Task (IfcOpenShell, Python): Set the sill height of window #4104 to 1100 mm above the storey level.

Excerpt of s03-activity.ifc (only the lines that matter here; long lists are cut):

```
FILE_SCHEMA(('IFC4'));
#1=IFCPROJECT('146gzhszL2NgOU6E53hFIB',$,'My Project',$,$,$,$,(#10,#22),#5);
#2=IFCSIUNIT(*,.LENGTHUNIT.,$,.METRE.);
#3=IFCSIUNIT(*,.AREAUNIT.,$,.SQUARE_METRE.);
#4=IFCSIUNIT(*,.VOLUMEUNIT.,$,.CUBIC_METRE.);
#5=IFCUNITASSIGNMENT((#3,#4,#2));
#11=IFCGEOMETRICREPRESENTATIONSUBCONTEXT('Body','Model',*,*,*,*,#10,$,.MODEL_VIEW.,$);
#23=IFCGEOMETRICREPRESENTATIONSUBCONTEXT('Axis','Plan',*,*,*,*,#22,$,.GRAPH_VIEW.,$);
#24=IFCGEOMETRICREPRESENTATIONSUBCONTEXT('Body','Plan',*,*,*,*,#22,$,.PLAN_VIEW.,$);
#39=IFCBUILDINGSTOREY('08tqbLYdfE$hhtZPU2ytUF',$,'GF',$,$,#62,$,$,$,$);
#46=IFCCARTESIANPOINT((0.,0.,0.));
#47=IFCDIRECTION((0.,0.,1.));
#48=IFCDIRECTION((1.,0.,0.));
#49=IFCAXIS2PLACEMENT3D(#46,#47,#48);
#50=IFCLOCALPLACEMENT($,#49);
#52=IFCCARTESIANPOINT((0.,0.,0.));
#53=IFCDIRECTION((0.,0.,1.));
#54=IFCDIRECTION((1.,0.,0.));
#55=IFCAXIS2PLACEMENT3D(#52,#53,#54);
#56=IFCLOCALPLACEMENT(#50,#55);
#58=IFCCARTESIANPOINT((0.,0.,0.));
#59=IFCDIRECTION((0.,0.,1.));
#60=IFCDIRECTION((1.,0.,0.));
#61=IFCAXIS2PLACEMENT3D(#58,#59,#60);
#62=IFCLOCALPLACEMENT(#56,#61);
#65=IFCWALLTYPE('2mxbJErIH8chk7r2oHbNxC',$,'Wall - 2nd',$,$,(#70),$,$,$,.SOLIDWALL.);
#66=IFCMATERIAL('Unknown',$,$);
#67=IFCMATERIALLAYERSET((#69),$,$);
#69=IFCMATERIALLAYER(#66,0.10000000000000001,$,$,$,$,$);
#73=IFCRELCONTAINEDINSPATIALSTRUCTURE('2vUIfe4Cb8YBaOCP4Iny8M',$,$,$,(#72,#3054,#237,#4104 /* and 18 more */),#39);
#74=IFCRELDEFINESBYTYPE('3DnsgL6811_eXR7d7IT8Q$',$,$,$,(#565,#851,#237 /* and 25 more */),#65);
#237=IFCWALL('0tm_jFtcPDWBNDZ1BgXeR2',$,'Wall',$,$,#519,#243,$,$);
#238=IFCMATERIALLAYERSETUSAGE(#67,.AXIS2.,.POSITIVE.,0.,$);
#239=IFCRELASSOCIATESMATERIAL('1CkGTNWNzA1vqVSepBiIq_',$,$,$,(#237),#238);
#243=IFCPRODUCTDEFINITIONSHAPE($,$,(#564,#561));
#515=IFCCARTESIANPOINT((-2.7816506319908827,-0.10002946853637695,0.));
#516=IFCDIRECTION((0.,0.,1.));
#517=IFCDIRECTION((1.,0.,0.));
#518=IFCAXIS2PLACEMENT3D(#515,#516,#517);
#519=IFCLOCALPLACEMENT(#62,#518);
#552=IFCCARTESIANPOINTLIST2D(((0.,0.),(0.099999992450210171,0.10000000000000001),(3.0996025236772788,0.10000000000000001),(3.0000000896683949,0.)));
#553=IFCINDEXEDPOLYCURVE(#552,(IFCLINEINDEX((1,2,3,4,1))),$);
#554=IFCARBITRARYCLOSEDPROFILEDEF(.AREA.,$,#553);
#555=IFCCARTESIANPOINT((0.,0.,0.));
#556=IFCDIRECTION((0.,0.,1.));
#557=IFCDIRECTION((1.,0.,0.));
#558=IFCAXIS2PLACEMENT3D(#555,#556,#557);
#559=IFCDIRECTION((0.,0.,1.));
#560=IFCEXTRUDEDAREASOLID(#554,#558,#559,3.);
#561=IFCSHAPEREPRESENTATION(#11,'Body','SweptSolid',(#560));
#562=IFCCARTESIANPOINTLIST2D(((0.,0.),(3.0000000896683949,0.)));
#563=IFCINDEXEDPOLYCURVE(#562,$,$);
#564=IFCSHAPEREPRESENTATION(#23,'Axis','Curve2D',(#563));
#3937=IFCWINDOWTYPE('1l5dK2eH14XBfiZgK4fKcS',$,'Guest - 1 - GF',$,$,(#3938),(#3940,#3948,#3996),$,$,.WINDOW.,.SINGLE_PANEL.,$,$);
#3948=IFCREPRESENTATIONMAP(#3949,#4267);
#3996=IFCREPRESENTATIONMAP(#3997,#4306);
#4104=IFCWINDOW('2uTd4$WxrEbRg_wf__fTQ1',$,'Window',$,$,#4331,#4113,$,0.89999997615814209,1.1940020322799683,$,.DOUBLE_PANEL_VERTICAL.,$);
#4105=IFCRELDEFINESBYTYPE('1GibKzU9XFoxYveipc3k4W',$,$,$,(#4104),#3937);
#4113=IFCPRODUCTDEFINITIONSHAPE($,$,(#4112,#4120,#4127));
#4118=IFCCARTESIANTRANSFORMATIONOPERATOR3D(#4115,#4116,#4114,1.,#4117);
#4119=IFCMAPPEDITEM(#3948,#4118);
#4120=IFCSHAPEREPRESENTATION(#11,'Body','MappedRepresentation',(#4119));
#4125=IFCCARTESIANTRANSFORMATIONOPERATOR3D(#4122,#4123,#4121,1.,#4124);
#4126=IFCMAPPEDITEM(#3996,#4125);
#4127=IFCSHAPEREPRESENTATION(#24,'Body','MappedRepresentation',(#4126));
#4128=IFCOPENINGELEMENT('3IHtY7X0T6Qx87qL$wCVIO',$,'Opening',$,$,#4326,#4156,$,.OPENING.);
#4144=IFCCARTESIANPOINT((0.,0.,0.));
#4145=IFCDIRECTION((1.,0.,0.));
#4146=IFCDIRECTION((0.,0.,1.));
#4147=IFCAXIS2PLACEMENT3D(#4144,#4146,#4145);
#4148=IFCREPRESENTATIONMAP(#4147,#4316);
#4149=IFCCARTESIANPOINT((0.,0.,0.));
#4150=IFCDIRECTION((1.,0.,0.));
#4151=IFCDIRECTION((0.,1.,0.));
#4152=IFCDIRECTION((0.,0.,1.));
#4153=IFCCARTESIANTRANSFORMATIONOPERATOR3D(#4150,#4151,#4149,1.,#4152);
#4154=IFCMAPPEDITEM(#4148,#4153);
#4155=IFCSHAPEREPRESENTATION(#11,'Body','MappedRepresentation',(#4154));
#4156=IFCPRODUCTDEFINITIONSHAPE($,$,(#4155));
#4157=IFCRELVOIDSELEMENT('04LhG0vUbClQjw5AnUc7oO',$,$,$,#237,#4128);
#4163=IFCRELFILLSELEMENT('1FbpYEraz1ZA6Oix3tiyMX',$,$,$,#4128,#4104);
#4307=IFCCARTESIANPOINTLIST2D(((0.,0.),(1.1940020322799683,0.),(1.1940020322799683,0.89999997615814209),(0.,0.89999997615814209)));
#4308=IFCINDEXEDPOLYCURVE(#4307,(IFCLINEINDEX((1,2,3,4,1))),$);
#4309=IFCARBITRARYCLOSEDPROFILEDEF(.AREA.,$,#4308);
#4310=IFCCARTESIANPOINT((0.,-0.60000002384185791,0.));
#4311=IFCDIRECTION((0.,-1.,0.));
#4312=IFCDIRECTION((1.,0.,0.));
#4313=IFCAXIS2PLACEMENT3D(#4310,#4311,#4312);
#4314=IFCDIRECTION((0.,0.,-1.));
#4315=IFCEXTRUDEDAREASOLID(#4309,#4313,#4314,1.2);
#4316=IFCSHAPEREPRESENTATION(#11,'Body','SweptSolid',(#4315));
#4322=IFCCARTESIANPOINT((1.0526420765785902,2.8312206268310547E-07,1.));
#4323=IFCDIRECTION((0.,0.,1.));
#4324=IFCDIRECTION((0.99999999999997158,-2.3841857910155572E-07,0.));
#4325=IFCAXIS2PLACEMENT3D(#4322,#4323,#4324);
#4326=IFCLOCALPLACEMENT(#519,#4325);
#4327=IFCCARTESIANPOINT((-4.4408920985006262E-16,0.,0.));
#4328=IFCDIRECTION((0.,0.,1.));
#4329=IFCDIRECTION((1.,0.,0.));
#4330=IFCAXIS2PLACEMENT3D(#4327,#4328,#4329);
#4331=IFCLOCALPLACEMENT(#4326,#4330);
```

```python
import numpy as np
import ifcopenshell
import ifcopenshell.api.geometry
import ifcopenshell.geom
import ifcopenshell.util.element
import ifcopenshell.util.placement
import ifcopenshell.util.shape
import ifcopenshell.util.unit

model = ifcopenshell.open("s03-activity.ifc")
unit_scale = ifcopenshell.util.unit.calculate_unit_scale(model)

window = model.by_guid("2uTd4$WxrEbRg_wf__fTQ1")
opening = window.FillsVoids[0].RelatingOpeningElement
storey = ifcopenshell.util.element.get_container(window, ifc_class="IfcBuildingStorey")
level = ifcopenshell.util.placement.get_local_placement(storey.ObjectPlacement)[2, 3]

# The opening's origin need not be at the sill, so measure its lowest point.
shape = ifcopenshell.geom.create_shape(ifcopenshell.geom.settings(), opening)
bottom = ifcopenshell.util.shape.get_shape_bottom_elevation(shape, shape.geometry) / unit_scale
dz = level + 1.1 / unit_scale - bottom

shift = np.array([0.0, 0.0, dz])
# The window is placed relative to its opening, so it follows when the opening moves.
matrix = ifcopenshell.util.placement.get_local_placement(opening.ObjectPlacement)
matrix[:3, 3] += shift
ifcopenshell.api.geometry.edit_object_placement(
    model, product=opening, matrix=matrix, is_si=False, should_transform_children=True
)

print(f"moved by {dz * unit_scale:+.3f} m")

model.write("s03-activity-out.ifc")
```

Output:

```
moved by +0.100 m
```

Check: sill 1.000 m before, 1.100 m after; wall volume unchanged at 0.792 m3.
